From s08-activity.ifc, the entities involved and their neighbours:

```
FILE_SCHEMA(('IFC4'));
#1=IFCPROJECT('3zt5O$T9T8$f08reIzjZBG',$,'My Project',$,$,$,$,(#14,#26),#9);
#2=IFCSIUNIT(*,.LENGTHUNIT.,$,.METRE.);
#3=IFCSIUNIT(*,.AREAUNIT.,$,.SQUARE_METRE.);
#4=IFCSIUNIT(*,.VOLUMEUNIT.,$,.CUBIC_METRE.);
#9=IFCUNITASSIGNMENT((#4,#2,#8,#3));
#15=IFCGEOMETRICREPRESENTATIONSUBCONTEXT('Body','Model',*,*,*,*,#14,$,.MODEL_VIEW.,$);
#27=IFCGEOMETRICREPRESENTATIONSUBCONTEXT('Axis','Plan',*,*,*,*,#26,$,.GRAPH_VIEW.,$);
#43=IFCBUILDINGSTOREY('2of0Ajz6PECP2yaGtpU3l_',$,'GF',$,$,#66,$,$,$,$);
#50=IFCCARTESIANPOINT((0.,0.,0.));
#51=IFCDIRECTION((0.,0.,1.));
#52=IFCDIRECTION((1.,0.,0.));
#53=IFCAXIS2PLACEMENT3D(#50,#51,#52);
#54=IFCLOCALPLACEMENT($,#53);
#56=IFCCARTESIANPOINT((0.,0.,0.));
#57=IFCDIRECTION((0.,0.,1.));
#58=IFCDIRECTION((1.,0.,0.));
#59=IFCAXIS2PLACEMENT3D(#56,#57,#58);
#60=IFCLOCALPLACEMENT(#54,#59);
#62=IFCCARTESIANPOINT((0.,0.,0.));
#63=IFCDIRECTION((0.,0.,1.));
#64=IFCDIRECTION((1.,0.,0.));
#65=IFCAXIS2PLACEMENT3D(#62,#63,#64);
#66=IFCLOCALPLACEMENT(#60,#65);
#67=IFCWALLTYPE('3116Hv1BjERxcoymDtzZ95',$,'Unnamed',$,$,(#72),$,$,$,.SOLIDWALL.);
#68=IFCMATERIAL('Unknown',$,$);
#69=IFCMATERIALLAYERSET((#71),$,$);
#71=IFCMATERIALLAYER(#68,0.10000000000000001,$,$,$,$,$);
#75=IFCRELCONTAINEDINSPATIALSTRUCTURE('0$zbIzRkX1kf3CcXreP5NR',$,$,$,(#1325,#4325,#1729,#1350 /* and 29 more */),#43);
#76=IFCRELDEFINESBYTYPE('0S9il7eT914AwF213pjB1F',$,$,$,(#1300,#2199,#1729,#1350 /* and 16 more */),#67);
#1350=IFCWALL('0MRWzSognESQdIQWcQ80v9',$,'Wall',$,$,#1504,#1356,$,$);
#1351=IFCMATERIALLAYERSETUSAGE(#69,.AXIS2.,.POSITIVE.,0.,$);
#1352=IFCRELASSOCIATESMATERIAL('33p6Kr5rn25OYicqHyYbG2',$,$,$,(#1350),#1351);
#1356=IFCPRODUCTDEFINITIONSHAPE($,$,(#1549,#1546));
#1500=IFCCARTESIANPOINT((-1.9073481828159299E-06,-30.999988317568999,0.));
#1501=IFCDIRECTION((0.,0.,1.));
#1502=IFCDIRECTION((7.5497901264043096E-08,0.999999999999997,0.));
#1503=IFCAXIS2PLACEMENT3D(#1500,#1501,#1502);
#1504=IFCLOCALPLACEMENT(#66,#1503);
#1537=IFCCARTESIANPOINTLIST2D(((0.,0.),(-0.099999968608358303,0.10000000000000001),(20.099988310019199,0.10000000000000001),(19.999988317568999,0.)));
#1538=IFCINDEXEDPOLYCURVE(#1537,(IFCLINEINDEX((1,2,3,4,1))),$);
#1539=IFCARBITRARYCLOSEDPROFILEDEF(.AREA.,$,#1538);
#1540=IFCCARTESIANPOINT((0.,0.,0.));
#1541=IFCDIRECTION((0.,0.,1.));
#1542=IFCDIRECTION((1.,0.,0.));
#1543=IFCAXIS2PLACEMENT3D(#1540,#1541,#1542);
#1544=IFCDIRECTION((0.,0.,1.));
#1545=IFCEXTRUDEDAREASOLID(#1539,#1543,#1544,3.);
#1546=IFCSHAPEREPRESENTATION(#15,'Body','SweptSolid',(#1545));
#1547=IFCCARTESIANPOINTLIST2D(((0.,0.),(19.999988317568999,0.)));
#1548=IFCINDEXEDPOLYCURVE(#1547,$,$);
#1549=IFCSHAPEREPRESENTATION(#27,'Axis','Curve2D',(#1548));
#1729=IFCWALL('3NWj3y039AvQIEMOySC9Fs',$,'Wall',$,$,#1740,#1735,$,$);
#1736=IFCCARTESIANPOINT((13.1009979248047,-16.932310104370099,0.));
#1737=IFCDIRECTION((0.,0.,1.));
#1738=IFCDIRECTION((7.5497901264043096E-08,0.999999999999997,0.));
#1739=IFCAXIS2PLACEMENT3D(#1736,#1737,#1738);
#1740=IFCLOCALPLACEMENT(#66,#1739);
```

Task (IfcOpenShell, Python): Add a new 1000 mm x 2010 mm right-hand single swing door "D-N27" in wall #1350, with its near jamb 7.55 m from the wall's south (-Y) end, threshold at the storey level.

```python
import numpy as np
import ifcopenshell
import ifcopenshell.api.feature
import ifcopenshell.api.geometry
import ifcopenshell.api.root
import ifcopenshell.api.spatial
import ifcopenshell.geom
import ifcopenshell.util.element
import ifcopenshell.util.placement
import ifcopenshell.util.representation
import ifcopenshell.util.shape
import ifcopenshell.util.unit

model = ifcopenshell.open("s08-activity.ifc")
unit_scale = ifcopenshell.util.unit.calculate_unit_scale(model)
settings = ifcopenshell.geom.settings()


def volume(element):
    """Net volume in cubic metres, openings subtracted."""
    shape = ifcopenshell.geom.create_shape(settings, element)
    return ifcopenshell.util.shape.get_volume(shape.geometry)


wall = model.by_guid("0MRWzSognESQdIQWcQ80v9")
storey = ifcopenshell.util.element.get_container(wall, ifc_class="IfcBuildingStorey")
context = ifcopenshell.util.representation.get_context(model, "Model", "Body", "MODEL_VIEW")
before = volume(wall)

width, height, from_end, sill = 1, 2.01, 7.55, 0.0  # metres

# The wall runs along its own X axis, and the end named is its -X end.
wall_shape = ifcopenshell.geom.create_shape(settings, wall)
x, y, z = ifcopenshell.util.shape.get_vertices(wall_shape.geometry).T
start = x.min() + from_end
face, thickness = float(y.min()), float(y.max() - y.min())
wall_matrix = ifcopenshell.util.placement.get_local_placement(wall.ObjectPlacement)
level = ifcopenshell.util.placement.get_local_placement(storey.ObjectPlacement)[2, 3]


def in_wall(x, y):
    """Placement at x, y metres in the wall's axes, at sill height."""
    matrix = wall_matrix.copy()
    matrix[:, 3] = wall_matrix @ np.array([x / unit_scale, y / unit_scale, 0.0, 1.0])
    matrix[2, 3] = level + sill / unit_scale
    return matrix


# Opening: a box that overshoots both wall faces by 50 mm.
opening = ifcopenshell.api.root.create_entity(model, ifc_class="IfcOpeningElement", predefined_type="OPENING")
box = ifcopenshell.api.geometry.add_wall_representation(
    model, context=context, length=width, height=height, thickness=thickness + 0.1
)
ifcopenshell.api.geometry.assign_representation(model, product=opening, representation=box)
ifcopenshell.api.geometry.edit_object_placement(model, product=opening, matrix=in_wall(start, face - 0.05), is_si=False)
ifcopenshell.api.feature.add_feature(model, feature=opening, element=wall)

door = ifcopenshell.api.root.create_entity(model, ifc_class="IfcDoor", name="D-N27", predefined_type="DOOR")
door.OverallWidth, door.OverallHeight = width / unit_scale, height / unit_scale
door.OperationType = "SINGLE_SWING_RIGHT"
body = ifcopenshell.api.geometry.add_door_representation(
    model,
    context=context,
    overall_width=door.OverallWidth,
    overall_height=door.OverallHeight,
    operation_type="SINGLE_SWING_RIGHT",
    lining_properties={"LiningDepth": thickness / unit_scale, "ThresholdDepth": thickness / unit_scale},
)
ifcopenshell.api.geometry.assign_representation(model, product=door, representation=body)
ifcopenshell.api.spatial.assign_container(model, products=[door], relating_structure=storey)
ifcopenshell.api.feature.add_filling(model, opening=opening, element=door)

# The lining spans the wall, so the door starts at the wall face.
ifcopenshell.api.geometry.edit_object_placement(model, product=door, matrix=in_wall(start, face), is_si=False)

after = volume(wall)

print(f"wall volume {before:.3f} -> {after:.3f} m3")

model.write("s08-activity_v2.ifc")
```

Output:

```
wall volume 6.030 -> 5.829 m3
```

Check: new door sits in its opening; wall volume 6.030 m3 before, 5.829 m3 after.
